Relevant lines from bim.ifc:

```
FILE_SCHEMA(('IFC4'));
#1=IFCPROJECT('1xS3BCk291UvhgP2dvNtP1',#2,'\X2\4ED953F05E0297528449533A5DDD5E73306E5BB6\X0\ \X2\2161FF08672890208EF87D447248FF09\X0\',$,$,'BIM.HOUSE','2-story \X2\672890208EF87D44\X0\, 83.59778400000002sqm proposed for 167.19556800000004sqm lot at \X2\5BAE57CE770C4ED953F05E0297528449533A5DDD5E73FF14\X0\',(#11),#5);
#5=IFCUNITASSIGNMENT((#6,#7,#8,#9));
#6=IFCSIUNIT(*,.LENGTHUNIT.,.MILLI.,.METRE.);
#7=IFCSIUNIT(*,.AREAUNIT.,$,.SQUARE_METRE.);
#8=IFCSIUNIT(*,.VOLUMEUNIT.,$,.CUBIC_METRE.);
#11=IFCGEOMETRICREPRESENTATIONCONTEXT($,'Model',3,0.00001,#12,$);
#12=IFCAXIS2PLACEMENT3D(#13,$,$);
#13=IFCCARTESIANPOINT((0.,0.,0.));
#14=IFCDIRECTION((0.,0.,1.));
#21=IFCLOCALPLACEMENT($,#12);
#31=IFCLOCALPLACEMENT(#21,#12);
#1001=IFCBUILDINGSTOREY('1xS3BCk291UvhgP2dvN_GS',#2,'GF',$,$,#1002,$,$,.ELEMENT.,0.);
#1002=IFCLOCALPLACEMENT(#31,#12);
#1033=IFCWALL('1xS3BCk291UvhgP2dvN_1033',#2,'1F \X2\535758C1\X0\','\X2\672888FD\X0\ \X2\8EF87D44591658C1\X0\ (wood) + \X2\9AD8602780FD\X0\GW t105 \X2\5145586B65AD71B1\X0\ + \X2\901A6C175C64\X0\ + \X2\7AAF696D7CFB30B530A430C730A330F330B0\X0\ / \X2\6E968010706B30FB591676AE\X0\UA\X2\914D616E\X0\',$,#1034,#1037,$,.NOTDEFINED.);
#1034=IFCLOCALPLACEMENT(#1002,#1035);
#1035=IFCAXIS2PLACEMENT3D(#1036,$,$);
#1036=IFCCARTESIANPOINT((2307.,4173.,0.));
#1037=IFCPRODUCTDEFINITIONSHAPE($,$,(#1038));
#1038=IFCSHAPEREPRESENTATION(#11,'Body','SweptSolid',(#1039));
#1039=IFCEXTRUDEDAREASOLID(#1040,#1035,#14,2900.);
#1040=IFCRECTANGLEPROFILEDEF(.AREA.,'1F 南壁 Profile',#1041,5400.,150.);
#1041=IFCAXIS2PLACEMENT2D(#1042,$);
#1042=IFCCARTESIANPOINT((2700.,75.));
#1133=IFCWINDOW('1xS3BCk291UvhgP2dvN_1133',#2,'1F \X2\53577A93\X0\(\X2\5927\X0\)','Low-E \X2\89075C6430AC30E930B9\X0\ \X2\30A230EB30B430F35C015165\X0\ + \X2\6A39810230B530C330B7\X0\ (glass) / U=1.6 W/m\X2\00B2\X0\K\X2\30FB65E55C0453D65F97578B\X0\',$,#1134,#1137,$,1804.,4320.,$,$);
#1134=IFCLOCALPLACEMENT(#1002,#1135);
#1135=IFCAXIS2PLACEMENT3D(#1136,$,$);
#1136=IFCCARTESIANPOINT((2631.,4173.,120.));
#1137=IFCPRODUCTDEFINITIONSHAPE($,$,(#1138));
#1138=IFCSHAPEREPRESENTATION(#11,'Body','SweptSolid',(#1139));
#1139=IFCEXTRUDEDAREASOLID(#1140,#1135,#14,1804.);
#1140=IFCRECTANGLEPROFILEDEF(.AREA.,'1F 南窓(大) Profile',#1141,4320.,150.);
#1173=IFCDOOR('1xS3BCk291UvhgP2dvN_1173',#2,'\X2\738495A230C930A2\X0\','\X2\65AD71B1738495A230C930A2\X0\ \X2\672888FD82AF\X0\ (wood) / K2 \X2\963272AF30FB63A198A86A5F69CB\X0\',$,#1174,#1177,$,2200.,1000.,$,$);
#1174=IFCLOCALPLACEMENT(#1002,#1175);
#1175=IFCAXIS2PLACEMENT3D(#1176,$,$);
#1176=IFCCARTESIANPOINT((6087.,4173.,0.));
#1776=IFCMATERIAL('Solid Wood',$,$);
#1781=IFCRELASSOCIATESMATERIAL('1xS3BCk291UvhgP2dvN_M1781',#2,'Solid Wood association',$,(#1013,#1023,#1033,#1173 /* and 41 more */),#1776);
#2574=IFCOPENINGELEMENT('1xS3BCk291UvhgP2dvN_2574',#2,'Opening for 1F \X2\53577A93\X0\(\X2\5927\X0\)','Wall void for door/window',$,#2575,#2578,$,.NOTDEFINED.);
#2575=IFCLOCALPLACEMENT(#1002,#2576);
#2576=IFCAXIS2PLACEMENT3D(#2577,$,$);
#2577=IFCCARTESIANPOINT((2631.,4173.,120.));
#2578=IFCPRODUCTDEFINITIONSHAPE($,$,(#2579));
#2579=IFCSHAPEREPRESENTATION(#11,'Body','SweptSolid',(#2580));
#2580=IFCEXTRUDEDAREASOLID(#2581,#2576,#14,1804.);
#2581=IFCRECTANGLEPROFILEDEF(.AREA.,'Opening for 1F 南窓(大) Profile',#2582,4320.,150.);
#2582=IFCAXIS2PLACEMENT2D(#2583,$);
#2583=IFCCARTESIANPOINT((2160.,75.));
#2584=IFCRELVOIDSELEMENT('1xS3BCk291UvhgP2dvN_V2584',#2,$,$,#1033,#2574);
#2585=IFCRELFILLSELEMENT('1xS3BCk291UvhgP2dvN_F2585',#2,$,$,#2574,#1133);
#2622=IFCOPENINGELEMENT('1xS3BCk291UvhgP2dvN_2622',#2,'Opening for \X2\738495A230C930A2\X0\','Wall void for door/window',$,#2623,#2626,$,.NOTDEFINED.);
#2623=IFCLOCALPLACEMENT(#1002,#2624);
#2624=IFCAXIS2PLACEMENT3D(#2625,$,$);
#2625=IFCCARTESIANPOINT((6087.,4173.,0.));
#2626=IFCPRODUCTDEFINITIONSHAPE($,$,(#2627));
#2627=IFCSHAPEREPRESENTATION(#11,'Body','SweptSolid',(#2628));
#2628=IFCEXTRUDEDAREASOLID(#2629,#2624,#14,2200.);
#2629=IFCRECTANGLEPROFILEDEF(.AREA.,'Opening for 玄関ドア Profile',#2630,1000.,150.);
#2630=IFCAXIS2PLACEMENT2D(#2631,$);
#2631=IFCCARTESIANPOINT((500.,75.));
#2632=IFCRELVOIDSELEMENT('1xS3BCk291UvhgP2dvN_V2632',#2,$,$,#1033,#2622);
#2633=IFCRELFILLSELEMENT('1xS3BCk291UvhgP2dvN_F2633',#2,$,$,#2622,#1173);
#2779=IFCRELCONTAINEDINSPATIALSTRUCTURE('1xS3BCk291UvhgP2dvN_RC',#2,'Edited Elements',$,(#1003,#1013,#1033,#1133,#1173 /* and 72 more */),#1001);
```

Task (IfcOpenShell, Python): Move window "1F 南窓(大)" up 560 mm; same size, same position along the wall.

```python
import numpy as np
import ifcopenshell
import ifcopenshell.api.geometry
import ifcopenshell.util.placement
import ifcopenshell.util.unit

model = ifcopenshell.open("bim.ifc")
unit_scale = ifcopenshell.util.unit.calculate_unit_scale(model)

window = model.by_guid("1xS3BCk291UvhgP2dvN_1133")
opening = window.FillsVoids[0].RelatingOpeningElement
dz = 560.0

shift = np.array([0.0, 0.0, dz])
# The window is not placed relative to its opening, so move both.
for product in (opening, window):
    matrix = ifcopenshell.util.placement.get_local_placement(product.ObjectPlacement)
    matrix[:3, 3] += shift
    ifcopenshell.api.geometry.edit_object_placement(model, product=product, matrix=matrix, is_si=False)

print(f"moved by {dz * unit_scale:+.3f} m")

model.write("bim_updated.ifc")
```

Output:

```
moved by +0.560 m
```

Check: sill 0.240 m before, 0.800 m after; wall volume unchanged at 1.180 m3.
